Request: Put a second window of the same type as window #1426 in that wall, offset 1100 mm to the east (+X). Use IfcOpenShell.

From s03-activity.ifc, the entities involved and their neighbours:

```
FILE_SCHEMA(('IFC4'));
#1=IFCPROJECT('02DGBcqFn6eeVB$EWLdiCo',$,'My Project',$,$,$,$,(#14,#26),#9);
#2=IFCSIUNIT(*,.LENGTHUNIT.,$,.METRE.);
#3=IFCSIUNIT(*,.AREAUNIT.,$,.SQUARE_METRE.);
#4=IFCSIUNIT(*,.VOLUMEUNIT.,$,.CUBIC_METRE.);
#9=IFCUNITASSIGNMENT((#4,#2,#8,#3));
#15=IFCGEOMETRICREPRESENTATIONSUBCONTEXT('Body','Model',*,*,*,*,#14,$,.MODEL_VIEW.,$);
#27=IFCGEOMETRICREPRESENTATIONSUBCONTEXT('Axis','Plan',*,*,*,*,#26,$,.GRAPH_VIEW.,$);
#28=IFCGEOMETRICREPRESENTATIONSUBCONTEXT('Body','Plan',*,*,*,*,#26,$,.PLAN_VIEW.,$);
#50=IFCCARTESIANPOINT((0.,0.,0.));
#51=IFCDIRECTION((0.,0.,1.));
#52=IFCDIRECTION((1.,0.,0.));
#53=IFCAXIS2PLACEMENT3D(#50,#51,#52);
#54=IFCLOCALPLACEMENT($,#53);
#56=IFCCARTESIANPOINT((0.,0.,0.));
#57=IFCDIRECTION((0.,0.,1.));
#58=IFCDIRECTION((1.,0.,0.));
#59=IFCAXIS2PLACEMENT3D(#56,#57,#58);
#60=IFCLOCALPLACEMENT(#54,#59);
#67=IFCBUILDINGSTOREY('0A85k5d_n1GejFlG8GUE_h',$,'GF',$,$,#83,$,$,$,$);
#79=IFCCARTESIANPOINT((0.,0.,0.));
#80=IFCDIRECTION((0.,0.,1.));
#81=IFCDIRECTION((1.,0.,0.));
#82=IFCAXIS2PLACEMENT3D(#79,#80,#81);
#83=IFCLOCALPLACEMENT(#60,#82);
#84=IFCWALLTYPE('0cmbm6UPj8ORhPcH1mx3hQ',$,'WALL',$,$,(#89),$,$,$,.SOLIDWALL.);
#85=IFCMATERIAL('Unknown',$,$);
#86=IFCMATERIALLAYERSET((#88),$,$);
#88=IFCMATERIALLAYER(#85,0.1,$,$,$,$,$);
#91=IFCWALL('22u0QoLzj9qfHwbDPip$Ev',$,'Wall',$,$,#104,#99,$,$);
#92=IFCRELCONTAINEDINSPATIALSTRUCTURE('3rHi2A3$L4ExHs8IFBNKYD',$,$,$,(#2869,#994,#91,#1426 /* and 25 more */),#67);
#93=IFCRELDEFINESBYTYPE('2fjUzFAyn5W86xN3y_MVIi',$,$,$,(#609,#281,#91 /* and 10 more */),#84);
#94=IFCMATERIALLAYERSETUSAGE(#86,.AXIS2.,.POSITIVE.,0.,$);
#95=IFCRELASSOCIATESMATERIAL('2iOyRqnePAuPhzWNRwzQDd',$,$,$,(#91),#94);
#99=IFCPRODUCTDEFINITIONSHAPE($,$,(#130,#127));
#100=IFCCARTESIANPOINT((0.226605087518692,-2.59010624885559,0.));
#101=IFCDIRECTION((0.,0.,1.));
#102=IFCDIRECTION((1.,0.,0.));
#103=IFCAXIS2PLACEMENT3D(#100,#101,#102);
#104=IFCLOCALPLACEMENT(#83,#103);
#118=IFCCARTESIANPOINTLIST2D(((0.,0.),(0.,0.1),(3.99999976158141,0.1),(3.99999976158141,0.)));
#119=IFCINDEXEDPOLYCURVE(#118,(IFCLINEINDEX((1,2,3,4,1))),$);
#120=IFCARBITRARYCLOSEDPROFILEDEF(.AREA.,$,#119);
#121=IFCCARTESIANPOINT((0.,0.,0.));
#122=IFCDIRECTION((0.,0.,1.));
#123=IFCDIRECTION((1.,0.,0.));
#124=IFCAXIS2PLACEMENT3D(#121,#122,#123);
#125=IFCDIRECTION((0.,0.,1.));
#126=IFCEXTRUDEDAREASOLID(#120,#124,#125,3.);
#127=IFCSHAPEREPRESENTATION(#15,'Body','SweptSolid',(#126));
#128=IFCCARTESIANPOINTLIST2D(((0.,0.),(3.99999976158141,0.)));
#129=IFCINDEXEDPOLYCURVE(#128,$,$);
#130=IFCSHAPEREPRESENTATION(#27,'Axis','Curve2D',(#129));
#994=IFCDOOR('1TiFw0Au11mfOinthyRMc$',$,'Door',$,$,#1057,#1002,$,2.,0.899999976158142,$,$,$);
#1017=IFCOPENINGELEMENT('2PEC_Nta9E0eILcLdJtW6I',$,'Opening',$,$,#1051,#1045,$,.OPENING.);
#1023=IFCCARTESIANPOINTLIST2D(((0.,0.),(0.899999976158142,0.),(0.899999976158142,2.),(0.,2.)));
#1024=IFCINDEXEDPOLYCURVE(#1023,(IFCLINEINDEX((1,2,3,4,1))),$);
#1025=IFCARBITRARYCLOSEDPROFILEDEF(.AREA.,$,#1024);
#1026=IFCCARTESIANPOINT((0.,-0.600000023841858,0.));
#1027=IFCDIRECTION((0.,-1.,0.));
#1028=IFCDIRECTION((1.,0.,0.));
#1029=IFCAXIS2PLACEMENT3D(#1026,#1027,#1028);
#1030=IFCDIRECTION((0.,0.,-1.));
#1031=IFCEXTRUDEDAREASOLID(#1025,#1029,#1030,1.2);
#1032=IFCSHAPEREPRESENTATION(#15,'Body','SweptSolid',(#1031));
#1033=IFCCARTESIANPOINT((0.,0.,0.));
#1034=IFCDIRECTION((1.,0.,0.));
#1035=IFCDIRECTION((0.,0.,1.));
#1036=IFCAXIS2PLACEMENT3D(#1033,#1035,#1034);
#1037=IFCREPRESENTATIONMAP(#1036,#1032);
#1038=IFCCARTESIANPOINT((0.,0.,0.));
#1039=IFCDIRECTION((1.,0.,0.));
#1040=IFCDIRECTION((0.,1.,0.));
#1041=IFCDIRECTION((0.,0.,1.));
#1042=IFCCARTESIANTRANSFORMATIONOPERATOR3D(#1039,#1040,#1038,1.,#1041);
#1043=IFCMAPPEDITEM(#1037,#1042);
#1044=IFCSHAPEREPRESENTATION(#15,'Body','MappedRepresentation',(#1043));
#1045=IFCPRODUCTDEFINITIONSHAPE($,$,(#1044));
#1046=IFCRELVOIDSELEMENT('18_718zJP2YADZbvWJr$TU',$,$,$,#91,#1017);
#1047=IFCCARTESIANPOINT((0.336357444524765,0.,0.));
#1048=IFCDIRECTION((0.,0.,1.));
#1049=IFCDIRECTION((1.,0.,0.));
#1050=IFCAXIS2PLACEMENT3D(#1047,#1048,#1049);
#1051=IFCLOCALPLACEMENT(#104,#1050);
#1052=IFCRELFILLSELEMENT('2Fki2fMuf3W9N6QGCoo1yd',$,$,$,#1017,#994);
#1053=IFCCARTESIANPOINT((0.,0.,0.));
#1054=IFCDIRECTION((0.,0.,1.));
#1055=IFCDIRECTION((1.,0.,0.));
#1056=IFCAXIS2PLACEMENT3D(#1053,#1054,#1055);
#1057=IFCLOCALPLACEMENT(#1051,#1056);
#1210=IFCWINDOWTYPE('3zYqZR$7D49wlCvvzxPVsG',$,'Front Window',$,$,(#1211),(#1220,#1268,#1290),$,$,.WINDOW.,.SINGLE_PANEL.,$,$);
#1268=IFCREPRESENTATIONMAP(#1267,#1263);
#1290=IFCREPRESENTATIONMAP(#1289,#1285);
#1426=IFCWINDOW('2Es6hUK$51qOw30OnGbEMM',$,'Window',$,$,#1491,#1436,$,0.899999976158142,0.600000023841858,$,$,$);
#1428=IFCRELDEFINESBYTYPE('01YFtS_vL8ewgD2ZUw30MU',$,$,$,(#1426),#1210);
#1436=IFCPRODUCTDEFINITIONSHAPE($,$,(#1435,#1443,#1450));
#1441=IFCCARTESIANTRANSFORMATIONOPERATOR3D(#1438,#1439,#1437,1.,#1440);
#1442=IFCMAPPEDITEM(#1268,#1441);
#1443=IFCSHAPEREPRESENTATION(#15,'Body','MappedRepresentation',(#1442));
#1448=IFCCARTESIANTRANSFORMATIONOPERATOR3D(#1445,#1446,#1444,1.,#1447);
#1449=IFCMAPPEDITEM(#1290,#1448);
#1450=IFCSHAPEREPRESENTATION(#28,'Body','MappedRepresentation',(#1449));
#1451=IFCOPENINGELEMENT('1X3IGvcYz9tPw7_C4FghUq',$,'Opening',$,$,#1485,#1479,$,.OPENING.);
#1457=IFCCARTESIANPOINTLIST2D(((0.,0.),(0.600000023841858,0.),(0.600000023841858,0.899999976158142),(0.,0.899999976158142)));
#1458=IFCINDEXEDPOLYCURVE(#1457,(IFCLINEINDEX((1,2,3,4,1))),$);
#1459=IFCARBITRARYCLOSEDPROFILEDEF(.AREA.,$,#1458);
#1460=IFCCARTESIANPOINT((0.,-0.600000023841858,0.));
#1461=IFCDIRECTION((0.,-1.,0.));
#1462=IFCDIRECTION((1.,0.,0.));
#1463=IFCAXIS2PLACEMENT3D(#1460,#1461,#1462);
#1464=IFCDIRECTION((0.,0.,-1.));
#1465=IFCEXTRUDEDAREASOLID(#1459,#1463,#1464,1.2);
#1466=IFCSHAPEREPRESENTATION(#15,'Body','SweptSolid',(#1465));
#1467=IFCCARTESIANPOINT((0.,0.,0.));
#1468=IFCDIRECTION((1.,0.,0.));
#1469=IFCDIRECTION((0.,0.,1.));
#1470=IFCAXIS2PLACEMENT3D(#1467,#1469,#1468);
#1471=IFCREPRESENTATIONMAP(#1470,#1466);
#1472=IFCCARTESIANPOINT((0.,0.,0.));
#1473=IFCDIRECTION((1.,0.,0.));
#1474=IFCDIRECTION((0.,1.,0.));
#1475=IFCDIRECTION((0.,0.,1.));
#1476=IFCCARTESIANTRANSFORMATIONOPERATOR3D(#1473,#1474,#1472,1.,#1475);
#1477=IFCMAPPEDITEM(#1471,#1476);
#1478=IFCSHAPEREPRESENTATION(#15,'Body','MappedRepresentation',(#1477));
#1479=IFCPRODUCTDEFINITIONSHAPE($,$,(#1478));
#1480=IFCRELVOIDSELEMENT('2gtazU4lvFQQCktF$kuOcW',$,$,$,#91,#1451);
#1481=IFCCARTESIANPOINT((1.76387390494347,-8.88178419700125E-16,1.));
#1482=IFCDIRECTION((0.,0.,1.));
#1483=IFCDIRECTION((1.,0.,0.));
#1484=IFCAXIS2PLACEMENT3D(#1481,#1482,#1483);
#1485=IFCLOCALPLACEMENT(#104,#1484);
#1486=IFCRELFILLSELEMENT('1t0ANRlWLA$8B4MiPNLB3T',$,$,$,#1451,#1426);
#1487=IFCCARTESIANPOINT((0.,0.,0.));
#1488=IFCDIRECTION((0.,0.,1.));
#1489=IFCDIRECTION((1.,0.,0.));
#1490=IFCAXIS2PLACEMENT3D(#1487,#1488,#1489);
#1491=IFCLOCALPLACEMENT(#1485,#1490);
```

```python
import ifcopenshell
import ifcopenshell.api.feature
import ifcopenshell.api.geometry
import ifcopenshell.api.root
import ifcopenshell.geom
import ifcopenshell.util.element
import ifcopenshell.util.placement
import ifcopenshell.util.shape
import ifcopenshell.util.unit

model = ifcopenshell.open("s03-activity.ifc")
unit_scale = ifcopenshell.util.unit.calculate_unit_scale(model)
settings = ifcopenshell.geom.settings()


def volume(element):
    """Net volume in cubic metres, openings subtracted."""
    shape = ifcopenshell.geom.create_shape(settings, element)
    return ifcopenshell.util.shape.get_volume(shape.geometry)


window = model.by_guid("2Es6hUK$51qOw30OnGbEMM")
opening = window.FillsVoids[0].RelatingOpeningElement
wall = opening.VoidsElements[0].RelatingBuildingElement
before = volume(wall)
shift = ifcopenshell.util.placement.get_local_placement(wall.ObjectPlacement)[:3, 0] * 1.1 / unit_scale

# copy_class copies the void relationship, type, container and properties, but no geometry.
new_opening = ifcopenshell.api.root.copy_class(model, product=opening)
new_opening.Representation = ifcopenshell.util.element.copy_deep(
    model, opening.Representation, exclude=["IfcGeometricRepresentationContext", "IfcRepresentationMap"]
)
new_window = ifcopenshell.api.root.copy_class(model, product=window)
new_window.Representation = ifcopenshell.util.element.copy_deep(
    model, window.Representation, exclude=["IfcGeometricRepresentationContext", "IfcRepresentationMap"]
)
ifcopenshell.api.feature.add_filling(model, opening=new_opening, element=new_window)

for old, new in ((opening, new_opening), (window, new_window)):
    matrix = ifcopenshell.util.placement.get_local_placement(old.ObjectPlacement)
    matrix[:3, 3] += shift
    ifcopenshell.api.geometry.edit_object_placement(model, product=new, matrix=matrix, is_si=False)

after = volume(wall)

print(f"wall volume {before:.3f} -> {after:.3f} m3")

model.write("s03-activity_edited.ifc")
```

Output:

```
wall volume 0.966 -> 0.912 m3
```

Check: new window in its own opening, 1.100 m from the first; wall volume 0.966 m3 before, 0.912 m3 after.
